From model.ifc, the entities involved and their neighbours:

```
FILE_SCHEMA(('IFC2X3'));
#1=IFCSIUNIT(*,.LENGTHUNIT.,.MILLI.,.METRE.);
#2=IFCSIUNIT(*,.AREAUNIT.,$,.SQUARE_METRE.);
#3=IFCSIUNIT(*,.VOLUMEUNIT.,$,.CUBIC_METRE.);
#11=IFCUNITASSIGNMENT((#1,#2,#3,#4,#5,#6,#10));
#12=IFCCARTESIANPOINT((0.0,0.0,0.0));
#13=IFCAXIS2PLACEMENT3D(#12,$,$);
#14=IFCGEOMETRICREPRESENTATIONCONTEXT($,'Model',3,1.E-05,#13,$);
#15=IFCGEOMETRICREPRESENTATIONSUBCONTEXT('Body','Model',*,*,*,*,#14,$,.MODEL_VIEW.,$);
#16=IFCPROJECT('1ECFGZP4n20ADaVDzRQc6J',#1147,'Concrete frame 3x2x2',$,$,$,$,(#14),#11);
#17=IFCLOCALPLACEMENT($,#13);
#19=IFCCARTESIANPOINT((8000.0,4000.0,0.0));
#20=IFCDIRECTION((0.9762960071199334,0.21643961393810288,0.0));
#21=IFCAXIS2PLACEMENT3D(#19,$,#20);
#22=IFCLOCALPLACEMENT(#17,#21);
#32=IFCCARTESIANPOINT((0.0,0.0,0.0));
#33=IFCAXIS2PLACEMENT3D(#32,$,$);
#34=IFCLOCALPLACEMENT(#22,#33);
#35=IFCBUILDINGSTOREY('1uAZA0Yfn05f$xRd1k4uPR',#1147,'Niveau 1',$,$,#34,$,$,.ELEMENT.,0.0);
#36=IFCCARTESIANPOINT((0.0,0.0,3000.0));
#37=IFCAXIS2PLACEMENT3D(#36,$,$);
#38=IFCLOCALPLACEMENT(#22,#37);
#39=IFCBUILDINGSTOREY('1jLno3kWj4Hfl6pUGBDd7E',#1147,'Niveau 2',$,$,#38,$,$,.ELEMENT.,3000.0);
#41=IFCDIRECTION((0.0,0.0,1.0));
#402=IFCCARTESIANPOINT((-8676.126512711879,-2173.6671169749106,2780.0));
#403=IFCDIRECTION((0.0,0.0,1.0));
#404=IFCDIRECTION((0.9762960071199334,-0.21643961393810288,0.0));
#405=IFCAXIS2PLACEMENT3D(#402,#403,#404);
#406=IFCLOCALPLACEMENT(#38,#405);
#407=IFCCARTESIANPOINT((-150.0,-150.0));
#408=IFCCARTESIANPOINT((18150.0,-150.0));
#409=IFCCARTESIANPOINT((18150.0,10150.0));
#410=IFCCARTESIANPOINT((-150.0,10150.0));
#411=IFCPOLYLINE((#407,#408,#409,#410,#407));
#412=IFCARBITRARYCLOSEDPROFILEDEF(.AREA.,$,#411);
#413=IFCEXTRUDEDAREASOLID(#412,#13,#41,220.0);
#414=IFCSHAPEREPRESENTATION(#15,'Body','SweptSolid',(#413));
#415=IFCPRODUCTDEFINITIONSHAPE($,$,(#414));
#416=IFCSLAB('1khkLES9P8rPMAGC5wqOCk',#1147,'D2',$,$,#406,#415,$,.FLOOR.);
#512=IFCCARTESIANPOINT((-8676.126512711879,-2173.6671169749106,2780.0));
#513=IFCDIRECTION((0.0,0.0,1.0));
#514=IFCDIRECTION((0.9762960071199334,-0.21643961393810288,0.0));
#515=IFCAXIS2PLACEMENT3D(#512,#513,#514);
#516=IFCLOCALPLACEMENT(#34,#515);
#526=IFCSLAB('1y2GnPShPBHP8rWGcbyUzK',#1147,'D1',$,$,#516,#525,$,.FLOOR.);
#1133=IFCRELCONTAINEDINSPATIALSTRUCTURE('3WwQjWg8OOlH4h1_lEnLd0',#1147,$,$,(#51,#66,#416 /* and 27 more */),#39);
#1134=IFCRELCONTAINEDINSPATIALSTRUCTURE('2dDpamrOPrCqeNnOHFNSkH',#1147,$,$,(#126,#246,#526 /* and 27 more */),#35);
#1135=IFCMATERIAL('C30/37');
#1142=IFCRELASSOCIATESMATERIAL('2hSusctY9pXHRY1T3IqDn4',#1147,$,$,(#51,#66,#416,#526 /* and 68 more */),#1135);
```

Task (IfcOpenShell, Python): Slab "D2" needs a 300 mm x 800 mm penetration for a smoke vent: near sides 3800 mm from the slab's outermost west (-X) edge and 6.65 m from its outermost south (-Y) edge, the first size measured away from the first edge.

```python
import numpy as np
import ifcopenshell
import ifcopenshell.api.feature
import ifcopenshell.api.geometry
import ifcopenshell.api.root
import ifcopenshell.geom
import ifcopenshell.util.placement
import ifcopenshell.util.representation
import ifcopenshell.util.shape
import ifcopenshell.util.unit

model = ifcopenshell.open("model.ifc")
unit_scale = ifcopenshell.util.unit.calculate_unit_scale(model)
settings = ifcopenshell.geom.settings()


def volume(element):
    """Net volume in cubic metres, openings subtracted."""
    shape = ifcopenshell.geom.create_shape(settings, element)
    return ifcopenshell.util.shape.get_volume(shape.geometry)


slab = model.by_guid("1khkLES9P8rPMAGC5wqOCk")
before = volume(slab)

# Extent in the slab's own axes, in metres. The edges named are its -X and -Y sides.
slab_shape = ifcopenshell.geom.create_shape(settings, slab)
vertices = ifcopenshell.util.shape.get_vertices(slab_shape.geometry)
x_min, y_min, bottom = vertices.min(axis=0)
top = vertices[:, 2].max()

opening = ifcopenshell.api.root.create_entity(model, ifc_class="IfcOpeningElement", name="Smoke vent opening")
context = ifcopenshell.util.representation.get_context(model, "Model", "Body", "MODEL_VIEW")
width, depth = 0.3, 0.8
outline = [(0.0, 0.0), (width, 0.0), (width, depth), (0.0, depth), (0.0, 0.0)]
# Overshoot both faces by 50 mm so the cut is clean.
shape = ifcopenshell.api.geometry.add_slab_representation(
    model, context=context, depth=top - bottom + 0.1, polyline=outline
)
ifcopenshell.api.geometry.assign_representation(model, product=opening, representation=shape)

matrix = ifcopenshell.util.placement.get_local_placement(slab.ObjectPlacement)
matrix[:, 3] = matrix @ np.append(np.array([x_min + 3.8, y_min + 6.65, bottom - 0.05]) / unit_scale, 1.0)
ifcopenshell.api.geometry.edit_object_placement(model, product=opening, matrix=matrix, is_si=False)
ifcopenshell.api.feature.add_feature(model, feature=opening, element=slab)

after = volume(slab)

print(f"slab volume {before:.3f} -> {after:.3f} m3")

model.write("model-out.ifc")
```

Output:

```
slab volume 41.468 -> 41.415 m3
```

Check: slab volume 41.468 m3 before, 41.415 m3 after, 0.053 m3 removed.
